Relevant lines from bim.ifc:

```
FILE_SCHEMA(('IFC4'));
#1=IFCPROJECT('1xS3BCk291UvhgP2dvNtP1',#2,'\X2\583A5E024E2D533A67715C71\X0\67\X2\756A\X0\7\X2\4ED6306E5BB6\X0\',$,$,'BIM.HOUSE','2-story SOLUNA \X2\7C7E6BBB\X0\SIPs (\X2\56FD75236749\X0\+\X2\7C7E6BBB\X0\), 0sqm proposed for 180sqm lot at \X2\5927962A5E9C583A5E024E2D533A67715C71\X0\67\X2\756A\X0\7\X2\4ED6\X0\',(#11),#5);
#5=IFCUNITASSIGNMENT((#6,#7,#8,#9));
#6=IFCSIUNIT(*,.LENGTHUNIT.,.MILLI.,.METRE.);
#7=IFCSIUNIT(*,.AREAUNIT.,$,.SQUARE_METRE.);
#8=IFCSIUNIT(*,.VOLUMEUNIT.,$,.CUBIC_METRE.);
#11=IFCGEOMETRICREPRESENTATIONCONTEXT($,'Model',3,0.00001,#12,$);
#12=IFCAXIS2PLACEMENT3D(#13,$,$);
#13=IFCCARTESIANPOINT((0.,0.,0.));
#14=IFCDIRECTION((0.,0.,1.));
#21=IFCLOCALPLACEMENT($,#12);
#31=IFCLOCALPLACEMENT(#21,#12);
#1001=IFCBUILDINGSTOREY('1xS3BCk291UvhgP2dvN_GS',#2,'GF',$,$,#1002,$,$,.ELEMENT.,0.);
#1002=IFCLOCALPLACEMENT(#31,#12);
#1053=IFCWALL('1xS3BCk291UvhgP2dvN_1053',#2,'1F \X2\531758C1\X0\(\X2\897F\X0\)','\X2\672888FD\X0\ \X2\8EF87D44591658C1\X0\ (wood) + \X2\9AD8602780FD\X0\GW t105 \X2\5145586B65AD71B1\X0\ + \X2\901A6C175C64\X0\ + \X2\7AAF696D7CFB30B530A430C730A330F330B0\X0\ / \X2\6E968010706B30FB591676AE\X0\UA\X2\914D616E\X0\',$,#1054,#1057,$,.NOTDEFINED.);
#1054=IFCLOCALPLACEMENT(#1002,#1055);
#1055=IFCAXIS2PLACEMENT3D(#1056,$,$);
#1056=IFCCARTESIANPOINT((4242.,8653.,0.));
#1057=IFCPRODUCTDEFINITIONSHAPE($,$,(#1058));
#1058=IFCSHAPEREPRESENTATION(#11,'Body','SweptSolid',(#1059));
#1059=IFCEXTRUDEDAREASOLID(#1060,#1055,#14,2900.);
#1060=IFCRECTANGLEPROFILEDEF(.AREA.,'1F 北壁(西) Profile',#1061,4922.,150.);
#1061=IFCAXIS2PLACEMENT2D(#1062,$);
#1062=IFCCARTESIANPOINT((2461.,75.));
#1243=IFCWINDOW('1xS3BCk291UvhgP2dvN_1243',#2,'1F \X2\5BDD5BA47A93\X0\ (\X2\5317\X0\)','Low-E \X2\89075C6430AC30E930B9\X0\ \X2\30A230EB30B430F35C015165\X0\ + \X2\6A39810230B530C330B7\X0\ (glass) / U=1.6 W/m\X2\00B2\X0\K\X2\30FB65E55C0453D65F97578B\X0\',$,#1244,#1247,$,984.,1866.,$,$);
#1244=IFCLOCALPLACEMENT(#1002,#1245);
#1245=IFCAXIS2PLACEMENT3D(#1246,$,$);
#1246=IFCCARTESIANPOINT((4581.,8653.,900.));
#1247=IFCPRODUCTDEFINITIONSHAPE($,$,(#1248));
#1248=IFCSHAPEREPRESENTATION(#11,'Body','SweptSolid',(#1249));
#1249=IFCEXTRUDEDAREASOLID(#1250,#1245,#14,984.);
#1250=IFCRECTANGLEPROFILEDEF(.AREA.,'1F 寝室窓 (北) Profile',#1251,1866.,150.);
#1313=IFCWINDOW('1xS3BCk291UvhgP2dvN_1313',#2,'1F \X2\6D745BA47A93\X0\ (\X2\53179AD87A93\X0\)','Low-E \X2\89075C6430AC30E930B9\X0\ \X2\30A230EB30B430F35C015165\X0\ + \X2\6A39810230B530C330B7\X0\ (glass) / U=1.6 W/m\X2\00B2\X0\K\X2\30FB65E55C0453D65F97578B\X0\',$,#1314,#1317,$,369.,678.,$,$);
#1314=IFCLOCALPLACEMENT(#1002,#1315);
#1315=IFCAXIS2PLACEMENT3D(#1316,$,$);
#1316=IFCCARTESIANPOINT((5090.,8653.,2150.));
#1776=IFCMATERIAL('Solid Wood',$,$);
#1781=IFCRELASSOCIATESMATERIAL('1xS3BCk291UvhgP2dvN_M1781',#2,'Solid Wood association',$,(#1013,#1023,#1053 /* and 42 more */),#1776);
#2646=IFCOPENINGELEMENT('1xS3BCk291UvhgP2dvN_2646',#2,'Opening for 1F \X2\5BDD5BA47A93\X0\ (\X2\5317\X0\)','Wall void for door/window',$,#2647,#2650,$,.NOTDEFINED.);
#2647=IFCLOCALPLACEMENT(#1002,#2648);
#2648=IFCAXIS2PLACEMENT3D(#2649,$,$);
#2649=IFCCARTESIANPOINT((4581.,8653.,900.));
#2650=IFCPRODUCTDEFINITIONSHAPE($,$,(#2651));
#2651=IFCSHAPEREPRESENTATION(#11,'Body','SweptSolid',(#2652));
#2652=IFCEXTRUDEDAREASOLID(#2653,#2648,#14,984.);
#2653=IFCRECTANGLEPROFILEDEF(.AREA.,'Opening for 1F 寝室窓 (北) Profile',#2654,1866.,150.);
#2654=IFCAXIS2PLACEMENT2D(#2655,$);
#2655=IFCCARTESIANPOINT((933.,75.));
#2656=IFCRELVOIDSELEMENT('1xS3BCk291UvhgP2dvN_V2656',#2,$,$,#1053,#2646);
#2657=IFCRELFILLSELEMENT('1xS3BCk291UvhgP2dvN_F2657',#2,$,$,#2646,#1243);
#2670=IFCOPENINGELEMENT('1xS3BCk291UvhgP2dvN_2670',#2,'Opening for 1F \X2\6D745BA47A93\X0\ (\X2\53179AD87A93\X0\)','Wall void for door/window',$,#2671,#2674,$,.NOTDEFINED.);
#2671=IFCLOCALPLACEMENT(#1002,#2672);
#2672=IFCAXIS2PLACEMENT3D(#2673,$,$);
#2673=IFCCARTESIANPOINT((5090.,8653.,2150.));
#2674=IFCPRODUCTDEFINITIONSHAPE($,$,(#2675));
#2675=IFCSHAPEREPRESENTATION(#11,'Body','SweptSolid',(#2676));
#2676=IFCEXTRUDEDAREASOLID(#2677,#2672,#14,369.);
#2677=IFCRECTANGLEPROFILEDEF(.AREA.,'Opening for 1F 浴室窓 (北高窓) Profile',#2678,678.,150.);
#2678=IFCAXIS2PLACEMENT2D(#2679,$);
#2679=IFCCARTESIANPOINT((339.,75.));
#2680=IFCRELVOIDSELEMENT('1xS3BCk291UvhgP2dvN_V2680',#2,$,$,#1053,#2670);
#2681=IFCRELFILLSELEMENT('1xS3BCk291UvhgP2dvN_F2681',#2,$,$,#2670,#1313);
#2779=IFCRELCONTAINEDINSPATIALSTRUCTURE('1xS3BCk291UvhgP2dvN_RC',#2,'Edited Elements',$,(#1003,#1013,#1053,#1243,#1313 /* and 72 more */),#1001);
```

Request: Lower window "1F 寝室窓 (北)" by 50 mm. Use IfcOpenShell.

```python
import numpy as np
import ifcopenshell
import ifcopenshell.api.geometry
import ifcopenshell.util.placement
import ifcopenshell.util.unit

model = ifcopenshell.open("bim.ifc")
unit_scale = ifcopenshell.util.unit.calculate_unit_scale(model)

window = model.by_guid("1xS3BCk291UvhgP2dvN_1243")
opening = window.FillsVoids[0].RelatingOpeningElement
dz = -50.0

shift = np.array([0.0, 0.0, dz])
# The window is not placed relative to its opening, so move both.
for product in (opening, window):
    matrix = ifcopenshell.util.placement.get_local_placement(product.ObjectPlacement)
    matrix[:3, 3] += shift
    ifcopenshell.api.geometry.edit_object_placement(model, product=product, matrix=matrix, is_si=False)

print(f"moved by {dz * unit_scale:+.3f} m")

model.write("bim_updated.ifc")
```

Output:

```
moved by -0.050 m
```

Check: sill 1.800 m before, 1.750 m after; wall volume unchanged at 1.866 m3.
